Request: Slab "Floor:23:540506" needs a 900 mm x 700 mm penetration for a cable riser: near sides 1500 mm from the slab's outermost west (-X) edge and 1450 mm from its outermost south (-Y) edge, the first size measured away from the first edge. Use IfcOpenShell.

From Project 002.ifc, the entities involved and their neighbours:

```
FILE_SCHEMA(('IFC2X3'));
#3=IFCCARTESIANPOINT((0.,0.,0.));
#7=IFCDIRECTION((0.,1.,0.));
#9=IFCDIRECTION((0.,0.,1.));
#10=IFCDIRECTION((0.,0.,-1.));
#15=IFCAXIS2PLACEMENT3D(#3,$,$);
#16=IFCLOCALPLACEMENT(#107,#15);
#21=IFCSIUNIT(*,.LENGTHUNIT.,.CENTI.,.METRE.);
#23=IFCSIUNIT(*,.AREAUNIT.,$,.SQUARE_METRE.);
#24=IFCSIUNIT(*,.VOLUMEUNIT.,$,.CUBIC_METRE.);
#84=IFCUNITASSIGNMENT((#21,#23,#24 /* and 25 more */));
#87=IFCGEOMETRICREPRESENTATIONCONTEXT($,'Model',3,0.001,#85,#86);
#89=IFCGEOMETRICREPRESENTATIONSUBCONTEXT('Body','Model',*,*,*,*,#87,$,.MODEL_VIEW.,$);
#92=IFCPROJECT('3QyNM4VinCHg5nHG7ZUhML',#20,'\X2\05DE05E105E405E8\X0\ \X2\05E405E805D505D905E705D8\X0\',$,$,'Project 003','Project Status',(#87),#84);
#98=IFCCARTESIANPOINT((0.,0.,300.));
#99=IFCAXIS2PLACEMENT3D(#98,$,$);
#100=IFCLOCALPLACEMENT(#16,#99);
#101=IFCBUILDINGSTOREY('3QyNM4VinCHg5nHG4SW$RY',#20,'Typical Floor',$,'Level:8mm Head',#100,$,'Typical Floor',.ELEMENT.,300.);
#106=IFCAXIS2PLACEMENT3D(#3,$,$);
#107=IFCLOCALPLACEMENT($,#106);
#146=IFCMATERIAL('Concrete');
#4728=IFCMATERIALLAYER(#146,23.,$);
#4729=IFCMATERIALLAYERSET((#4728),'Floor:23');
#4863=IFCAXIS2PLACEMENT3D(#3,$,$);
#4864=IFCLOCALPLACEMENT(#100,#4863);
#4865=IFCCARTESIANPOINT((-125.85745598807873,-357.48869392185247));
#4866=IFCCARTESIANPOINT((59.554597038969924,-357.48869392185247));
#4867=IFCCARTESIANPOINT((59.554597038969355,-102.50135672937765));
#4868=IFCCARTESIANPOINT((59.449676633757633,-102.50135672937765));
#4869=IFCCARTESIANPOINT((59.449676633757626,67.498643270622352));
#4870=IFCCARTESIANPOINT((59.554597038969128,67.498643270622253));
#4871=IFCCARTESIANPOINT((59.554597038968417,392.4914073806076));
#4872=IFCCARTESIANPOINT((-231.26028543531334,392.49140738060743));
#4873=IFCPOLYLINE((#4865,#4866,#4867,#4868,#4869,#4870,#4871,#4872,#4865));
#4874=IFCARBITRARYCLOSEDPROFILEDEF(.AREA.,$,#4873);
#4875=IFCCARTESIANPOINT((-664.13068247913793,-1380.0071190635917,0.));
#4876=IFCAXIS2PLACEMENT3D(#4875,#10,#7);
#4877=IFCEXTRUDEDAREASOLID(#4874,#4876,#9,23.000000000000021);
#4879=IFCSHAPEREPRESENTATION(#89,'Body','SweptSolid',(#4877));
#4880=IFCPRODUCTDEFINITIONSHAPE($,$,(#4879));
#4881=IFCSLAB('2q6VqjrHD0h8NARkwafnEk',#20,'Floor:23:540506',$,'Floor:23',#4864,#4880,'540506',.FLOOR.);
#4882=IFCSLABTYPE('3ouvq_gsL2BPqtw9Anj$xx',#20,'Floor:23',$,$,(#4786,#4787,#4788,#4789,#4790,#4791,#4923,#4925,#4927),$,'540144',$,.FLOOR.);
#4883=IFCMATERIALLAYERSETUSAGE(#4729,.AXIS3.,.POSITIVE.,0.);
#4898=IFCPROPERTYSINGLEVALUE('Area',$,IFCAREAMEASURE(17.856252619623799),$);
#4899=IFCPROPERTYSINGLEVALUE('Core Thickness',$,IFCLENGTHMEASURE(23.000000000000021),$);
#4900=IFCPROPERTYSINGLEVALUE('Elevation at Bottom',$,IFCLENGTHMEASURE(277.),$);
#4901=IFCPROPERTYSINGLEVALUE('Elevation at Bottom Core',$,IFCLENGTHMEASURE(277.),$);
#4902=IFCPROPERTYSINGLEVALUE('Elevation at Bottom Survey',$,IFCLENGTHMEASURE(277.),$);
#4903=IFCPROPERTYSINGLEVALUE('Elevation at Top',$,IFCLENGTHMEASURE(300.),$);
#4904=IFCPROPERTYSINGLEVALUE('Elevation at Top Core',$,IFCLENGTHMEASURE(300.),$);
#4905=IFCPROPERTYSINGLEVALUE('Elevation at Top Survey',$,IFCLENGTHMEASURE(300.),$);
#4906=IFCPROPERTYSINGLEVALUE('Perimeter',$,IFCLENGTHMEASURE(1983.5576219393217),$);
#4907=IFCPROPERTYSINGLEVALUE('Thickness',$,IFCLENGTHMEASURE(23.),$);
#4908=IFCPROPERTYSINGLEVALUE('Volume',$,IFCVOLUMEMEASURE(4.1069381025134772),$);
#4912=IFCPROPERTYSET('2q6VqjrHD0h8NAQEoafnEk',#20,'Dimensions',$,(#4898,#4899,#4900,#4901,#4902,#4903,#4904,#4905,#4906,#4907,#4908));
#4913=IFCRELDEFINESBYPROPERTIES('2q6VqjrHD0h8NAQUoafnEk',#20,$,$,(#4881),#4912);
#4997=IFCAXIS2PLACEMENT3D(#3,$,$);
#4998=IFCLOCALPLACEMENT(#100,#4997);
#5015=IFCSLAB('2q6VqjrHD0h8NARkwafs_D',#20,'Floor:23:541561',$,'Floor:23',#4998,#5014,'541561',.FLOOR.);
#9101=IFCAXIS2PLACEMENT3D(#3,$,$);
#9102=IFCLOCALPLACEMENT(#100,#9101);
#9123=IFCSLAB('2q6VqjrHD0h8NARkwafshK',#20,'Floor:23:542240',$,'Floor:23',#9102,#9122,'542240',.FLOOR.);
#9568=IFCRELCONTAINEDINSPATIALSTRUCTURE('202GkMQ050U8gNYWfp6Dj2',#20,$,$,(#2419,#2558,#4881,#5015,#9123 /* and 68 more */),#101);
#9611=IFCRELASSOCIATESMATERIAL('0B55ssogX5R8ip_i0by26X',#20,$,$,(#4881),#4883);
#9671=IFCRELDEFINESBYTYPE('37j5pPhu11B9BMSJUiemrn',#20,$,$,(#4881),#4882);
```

```python
import numpy as np
import ifcopenshell
import ifcopenshell.api.feature
import ifcopenshell.api.geometry
import ifcopenshell.api.pset
import ifcopenshell.api.root
import ifcopenshell.geom
import ifcopenshell.util.element
import ifcopenshell.util.placement
import ifcopenshell.util.representation
import ifcopenshell.util.shape
import ifcopenshell.util.unit

model = ifcopenshell.open("Project 002.ifc")
unit_scale = ifcopenshell.util.unit.calculate_unit_scale(model)
area_scale = ifcopenshell.util.unit.calculate_unit_scale(model, "AREAUNIT")
volume_scale = ifcopenshell.util.unit.calculate_unit_scale(model, "VOLUMEUNIT")
settings = ifcopenshell.geom.settings()


def volume(element):
    """Net volume in cubic metres, openings subtracted."""
    shape = ifcopenshell.geom.create_shape(settings, element)
    return ifcopenshell.util.shape.get_volume(shape.geometry)


slab = model.by_id(4881)
before = volume(slab)

# Extent in the slab's own axes, in metres. The edges named are its -X and -Y sides.
slab_shape = ifcopenshell.geom.create_shape(settings, slab)
vertices = ifcopenshell.util.shape.get_vertices(slab_shape.geometry)
x_min, y_min, bottom = vertices.min(axis=0)
top = vertices[:, 2].max()

opening = ifcopenshell.api.root.create_entity(model, ifc_class="IfcOpeningElement", name="Cable riser opening")
context = ifcopenshell.util.representation.get_context(model, "Model", "Body", "MODEL_VIEW")
width, depth = 0.9, 0.7
outline = [(0.0, 0.0), (width, 0.0), (width, depth), (0.0, depth), (0.0, 0.0)]
# Overshoot both faces by 50 mm so the cut is clean.
shape = ifcopenshell.api.geometry.add_slab_representation(
    model, context=context, depth=top - bottom + 0.1, polyline=outline
)
ifcopenshell.api.geometry.assign_representation(model, product=opening, representation=shape)

matrix = ifcopenshell.util.placement.get_local_placement(slab.ObjectPlacement)
matrix[:, 3] = matrix @ np.append(np.array([x_min + 1.5, y_min + 1.45, bottom - 0.05]) / unit_scale, 1.0)
ifcopenshell.api.geometry.edit_object_placement(model, product=opening, matrix=matrix, is_si=False)
ifcopenshell.api.feature.add_feature(model, feature=opening, element=slab)

after = volume(slab)

# Update the slab's stored quantities.
pset = model.by_id(ifcopenshell.util.element.get_pset(slab, "Dimensions", should_inherit=False)["id"])
ifcopenshell.api.pset.edit_pset(model, pset=pset, properties={
    "Area": model.create_entity("IfcAreaMeasure", after / (top - bottom) / area_scale),
    "Volume": model.create_entity("IfcVolumeMeasure", after / volume_scale),
})

print(f"slab volume {before:.3f} -> {after:.3f} m3")

model.write("Project 002_rev.ifc")
```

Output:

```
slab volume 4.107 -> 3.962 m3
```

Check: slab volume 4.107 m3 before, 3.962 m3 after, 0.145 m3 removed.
